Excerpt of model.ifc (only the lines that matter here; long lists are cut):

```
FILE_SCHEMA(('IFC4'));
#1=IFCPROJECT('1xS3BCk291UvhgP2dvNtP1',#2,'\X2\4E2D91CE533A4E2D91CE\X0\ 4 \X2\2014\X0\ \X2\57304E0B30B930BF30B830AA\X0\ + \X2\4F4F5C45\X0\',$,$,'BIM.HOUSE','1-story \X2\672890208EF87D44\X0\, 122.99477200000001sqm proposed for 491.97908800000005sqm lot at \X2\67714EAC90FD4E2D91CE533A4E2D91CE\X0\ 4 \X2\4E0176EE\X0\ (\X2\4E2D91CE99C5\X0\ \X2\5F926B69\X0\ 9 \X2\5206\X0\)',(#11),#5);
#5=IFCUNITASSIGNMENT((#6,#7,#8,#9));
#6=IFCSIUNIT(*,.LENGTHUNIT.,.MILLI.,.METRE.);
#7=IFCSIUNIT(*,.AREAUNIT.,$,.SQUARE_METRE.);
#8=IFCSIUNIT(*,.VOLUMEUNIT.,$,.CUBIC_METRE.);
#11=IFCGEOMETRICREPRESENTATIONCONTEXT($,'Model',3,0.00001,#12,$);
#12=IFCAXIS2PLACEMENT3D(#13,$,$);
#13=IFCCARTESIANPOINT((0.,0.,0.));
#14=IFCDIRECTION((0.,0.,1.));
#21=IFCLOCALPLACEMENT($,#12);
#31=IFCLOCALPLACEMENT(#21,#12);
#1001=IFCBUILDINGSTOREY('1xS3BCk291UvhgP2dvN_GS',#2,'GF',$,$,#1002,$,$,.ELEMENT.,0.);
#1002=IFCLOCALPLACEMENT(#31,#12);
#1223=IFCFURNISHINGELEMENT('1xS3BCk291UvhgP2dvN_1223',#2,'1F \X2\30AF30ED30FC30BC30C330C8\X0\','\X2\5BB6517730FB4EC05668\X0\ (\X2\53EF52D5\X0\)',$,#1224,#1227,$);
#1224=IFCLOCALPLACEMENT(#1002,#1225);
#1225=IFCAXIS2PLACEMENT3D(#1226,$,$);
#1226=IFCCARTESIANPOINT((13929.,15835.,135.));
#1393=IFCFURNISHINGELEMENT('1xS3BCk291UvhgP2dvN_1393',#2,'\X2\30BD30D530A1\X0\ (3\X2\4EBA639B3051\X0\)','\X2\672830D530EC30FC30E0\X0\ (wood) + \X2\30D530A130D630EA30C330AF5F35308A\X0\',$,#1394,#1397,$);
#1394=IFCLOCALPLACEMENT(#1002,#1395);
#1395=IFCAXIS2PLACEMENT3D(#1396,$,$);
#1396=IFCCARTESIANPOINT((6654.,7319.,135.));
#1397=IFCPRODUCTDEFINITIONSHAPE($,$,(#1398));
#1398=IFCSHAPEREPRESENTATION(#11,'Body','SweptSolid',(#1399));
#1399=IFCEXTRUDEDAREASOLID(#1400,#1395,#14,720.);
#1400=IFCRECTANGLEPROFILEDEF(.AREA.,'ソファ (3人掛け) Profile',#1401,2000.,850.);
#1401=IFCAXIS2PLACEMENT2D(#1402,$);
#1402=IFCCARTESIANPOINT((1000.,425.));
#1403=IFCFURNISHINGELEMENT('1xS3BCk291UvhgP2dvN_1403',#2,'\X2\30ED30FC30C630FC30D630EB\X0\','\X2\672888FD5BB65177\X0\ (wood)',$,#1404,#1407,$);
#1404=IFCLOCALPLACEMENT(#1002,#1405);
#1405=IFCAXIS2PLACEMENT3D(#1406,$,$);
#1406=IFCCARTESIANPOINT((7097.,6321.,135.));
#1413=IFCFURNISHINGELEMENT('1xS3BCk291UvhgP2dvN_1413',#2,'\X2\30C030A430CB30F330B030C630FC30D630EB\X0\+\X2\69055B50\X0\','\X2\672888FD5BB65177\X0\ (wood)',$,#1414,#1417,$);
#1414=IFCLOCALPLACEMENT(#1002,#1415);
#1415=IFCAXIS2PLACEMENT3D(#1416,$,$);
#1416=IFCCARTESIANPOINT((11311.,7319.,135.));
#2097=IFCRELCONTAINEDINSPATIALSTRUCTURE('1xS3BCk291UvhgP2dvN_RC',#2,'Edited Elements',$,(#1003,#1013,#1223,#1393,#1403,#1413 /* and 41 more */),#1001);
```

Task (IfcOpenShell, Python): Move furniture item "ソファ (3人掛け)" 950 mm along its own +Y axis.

```python
import ifcopenshell
import ifcopenshell.api.geometry
import ifcopenshell.util.placement
import ifcopenshell.util.unit

model = ifcopenshell.open("model.ifc")
unit_scale = ifcopenshell.util.unit.calculate_unit_scale(model)

item = model.by_id(1393)
matrix = ifcopenshell.util.placement.get_local_placement(item.ObjectPlacement)
matrix[:3, 3] += matrix[:3, 1] * 0.95 / unit_scale
ifcopenshell.api.geometry.edit_object_placement(model, product=item, matrix=matrix, is_si=False)

print(ifcopenshell.util.placement.get_local_placement(item.ObjectPlacement).round(3) + 0.0)

model.write("model_rev.ifc")
```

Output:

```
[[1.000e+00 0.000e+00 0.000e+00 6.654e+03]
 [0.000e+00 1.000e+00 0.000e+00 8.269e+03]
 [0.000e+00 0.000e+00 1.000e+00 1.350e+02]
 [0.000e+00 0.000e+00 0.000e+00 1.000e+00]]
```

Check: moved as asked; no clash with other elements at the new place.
